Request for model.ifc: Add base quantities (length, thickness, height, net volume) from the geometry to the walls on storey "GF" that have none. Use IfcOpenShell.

First a look at what the model holds.

```python
import ifcopenshell
import ifcopenshell.util.element
import ifcopenshell.util.unit

model = ifcopenshell.open("model.ifc")
print(model.schema)
for unit_type in ("LENGTHUNIT", "AREAUNIT", "VOLUMEUNIT"):
    print(unit_type, ifcopenshell.util.unit.calculate_unit_scale(model, unit_type))
storey = next(s for s in model.by_type("IfcBuildingStorey") if s.Name == "GF")
walls = [e for e in ifcopenshell.util.element.get_decomposition(storey) if e.is_a("IfcWall")]
for e in sorted(walls, key=lambda e: e.id()):
    print(e.id(), e.is_a(), e.Name, list(ifcopenshell.util.element.get_psets(e, qtos_only=True)), sep=" | ")
```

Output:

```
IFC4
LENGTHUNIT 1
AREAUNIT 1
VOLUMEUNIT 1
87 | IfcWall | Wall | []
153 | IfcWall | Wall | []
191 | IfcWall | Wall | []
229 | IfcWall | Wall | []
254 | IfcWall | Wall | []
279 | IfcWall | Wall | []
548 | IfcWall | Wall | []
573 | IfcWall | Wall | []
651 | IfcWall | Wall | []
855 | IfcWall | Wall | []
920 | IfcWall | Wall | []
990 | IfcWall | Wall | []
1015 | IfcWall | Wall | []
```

```python
import ifcopenshell
import ifcopenshell.api.pset
import ifcopenshell.geom
import ifcopenshell.util.element
import ifcopenshell.util.shape
import ifcopenshell.util.unit

model = ifcopenshell.open("model.ifc")
unit_scale = ifcopenshell.util.unit.calculate_unit_scale(model)
volume_scale = ifcopenshell.util.unit.calculate_unit_scale(model, "VOLUMEUNIT")
settings = ifcopenshell.geom.settings()

storey = next(s for s in model.by_type("IfcBuildingStorey") if s.Name == "GF")
walls = [e for e in ifcopenshell.util.element.get_decomposition(storey) if e.is_a("IfcWall")]

for e in sorted(walls, key=lambda e: e.id()):
    if ifcopenshell.util.element.get_psets(e, qtos_only=True, should_inherit=False):
        continue
    # Geometry comes back in metres, in the element's own axes.
    shape = ifcopenshell.geom.create_shape(settings, e)
    values = {
        "Length": ifcopenshell.util.shape.get_x(shape.geometry) / unit_scale,
        "Width": ifcopenshell.util.shape.get_y(shape.geometry) / unit_scale,
        "Height": ifcopenshell.util.shape.get_z(shape.geometry) / unit_scale,
        "NetVolume": ifcopenshell.util.shape.get_volume(shape.geometry) / volume_scale,
    }
    qto = ifcopenshell.api.pset.add_qto(model, product=e, name="Qto_WallBaseQuantities")
    ifcopenshell.api.pset.edit_qto(model, qto=qto, properties=values)
    print(e.id(), {k: round(v, 3) for k, v in values.items()})

model.write("model-out.ifc")
```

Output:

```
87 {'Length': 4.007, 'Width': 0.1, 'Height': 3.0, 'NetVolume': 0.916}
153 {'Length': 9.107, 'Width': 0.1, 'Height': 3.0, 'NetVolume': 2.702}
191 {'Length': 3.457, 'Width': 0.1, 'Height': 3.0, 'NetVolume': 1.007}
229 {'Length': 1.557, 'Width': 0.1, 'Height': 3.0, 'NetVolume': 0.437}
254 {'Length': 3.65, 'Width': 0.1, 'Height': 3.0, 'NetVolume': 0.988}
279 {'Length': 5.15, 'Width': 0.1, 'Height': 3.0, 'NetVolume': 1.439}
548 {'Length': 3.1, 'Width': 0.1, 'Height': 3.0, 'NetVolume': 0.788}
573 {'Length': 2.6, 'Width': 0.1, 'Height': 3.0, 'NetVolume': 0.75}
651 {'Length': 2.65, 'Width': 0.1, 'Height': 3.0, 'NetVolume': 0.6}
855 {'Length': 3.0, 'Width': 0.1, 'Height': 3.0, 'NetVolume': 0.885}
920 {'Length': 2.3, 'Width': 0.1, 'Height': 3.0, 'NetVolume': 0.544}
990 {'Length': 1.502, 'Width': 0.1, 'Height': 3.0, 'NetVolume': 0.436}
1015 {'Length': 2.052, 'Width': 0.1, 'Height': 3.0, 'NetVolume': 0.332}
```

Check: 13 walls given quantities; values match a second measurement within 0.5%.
